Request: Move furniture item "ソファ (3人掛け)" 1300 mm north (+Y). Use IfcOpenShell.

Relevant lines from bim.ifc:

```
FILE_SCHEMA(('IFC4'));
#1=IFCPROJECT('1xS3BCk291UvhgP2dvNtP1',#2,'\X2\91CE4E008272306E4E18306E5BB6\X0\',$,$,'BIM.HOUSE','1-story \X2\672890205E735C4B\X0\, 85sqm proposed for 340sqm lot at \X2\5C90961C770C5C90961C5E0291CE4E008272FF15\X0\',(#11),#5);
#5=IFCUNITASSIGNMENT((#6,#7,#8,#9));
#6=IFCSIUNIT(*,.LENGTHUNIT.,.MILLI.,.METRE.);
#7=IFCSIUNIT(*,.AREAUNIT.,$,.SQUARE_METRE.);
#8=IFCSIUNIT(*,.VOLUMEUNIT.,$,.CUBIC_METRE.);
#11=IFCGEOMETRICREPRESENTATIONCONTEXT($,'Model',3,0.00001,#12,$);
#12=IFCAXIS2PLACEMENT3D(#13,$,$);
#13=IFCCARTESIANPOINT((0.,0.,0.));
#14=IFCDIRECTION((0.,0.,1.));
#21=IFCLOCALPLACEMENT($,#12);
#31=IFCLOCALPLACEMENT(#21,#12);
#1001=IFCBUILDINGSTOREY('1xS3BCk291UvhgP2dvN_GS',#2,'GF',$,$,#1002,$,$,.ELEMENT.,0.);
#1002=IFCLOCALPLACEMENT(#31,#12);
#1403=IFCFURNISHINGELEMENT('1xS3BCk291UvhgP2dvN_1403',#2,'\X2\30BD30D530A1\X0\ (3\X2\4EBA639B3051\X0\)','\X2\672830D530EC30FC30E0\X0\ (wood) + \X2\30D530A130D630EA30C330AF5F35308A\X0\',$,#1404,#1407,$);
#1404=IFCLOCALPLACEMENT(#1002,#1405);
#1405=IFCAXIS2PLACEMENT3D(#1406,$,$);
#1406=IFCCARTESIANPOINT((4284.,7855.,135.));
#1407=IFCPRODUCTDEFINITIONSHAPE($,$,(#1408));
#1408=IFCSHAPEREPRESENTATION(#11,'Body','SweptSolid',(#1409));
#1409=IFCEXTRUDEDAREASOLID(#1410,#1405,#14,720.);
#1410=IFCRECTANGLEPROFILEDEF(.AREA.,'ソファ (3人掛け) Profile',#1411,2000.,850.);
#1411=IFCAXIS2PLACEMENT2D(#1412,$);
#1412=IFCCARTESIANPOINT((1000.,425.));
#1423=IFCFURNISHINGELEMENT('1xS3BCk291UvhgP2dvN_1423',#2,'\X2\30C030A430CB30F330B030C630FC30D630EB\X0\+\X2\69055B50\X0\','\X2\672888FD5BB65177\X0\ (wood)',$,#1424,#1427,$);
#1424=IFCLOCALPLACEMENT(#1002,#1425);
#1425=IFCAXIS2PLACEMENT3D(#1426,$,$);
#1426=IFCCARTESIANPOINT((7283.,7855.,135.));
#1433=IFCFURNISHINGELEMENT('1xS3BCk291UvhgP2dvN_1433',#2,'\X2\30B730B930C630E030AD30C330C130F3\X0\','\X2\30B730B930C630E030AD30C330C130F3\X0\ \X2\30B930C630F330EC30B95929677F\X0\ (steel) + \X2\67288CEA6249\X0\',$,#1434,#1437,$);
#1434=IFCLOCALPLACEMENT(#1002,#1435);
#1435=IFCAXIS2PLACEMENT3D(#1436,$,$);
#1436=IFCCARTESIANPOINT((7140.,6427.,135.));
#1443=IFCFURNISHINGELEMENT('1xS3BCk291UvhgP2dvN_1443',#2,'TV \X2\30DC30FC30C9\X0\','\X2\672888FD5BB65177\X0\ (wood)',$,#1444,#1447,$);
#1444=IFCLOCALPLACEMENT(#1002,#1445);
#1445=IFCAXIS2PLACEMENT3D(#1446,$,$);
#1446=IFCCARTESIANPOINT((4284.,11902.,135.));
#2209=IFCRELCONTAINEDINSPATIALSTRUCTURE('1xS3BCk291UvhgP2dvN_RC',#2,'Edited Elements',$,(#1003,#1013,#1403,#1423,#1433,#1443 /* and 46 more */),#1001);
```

```python
import ifcopenshell
import ifcopenshell.api.geometry
import ifcopenshell.util.placement

model = ifcopenshell.open("bim.ifc")

item = model.by_guid("1xS3BCk291UvhgP2dvN_1403")
matrix = ifcopenshell.util.placement.get_local_placement(item.ObjectPlacement)
matrix[1, 3] += 1300.0
ifcopenshell.api.geometry.edit_object_placement(model, product=item, matrix=matrix, is_si=False)

print(ifcopenshell.util.placement.get_local_placement(item.ObjectPlacement).round(3) + 0.0)

model.write("bim_rev.ifc")
```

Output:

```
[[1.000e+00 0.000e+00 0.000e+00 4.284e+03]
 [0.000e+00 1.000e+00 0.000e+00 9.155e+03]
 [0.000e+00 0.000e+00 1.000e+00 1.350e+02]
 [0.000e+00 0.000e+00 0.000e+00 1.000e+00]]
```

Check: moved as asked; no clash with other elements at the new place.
